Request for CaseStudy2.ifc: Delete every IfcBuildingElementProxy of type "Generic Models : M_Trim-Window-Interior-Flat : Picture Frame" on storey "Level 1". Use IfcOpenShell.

First a look at what the model holds.

```python
import ifcopenshell
import ifcopenshell.util.element

model = ifcopenshell.open("CaseStudy2.ifc")
print(model.schema)
storey = next(s for s in model.by_type("IfcBuildingStorey") if s.Name == "Level 1")
proxies = [e for e in ifcopenshell.util.element.get_decomposition(storey) if e.is_a("IfcBuildingElementProxy")]
seen = {}
for e in proxies:
    element_type = ifcopenshell.util.element.get_type(e)
    name = element_type.Name if element_type not in (None, e) else None
    seen[name] = seen.get(name, 0) + 1
for name, count in sorted(seen.items(), key=str):
    print(count, "x", name)
```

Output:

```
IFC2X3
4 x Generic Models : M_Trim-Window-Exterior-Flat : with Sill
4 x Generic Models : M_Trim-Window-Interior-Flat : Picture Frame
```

```python
import ifcopenshell
import ifcopenshell.api.root
import ifcopenshell.util.element

model = ifcopenshell.open("CaseStudy2.ifc")

storey = next(s for s in model.by_type("IfcBuildingStorey") if s.Name == "Level 1")
proxies = [e for e in ifcopenshell.util.element.get_decomposition(storey) if e.is_a("IfcBuildingElementProxy")]
targets = [e for e in proxies if (t := ifcopenshell.util.element.get_type(e)) not in (None, e) and t.Name == "Generic Models : M_Trim-Window-Interior-Flat : Picture Frame"]

for e in targets:
    ifcopenshell.api.root.remove_product(model, product=e)
print(len(targets), "removed")

model.write("CaseStudy2-out.ifc")
```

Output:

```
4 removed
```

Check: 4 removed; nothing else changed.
